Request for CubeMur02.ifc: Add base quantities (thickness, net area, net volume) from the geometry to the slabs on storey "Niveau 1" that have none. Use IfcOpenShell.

First a look at what the model holds.

```python
import ifcopenshell
import ifcopenshell.util.element
import ifcopenshell.util.unit

model = ifcopenshell.open("CubeMur02.ifc")
print(model.schema)
for unit_type in ("LENGTHUNIT", "AREAUNIT", "VOLUMEUNIT"):
    print(unit_type, ifcopenshell.util.unit.calculate_unit_scale(model, unit_type))
storey = next(s for s in model.by_type("IfcBuildingStorey") if s.Name == "Niveau 1")
slabs = [e for e in ifcopenshell.util.element.get_decomposition(storey) if e.is_a("IfcSlab")]
for e in sorted(slabs, key=lambda e: e.id()):
    print(e.id(), e.is_a(), e.Name, list(ifcopenshell.util.element.get_psets(e, qtos_only=True)), sep=" | ")
```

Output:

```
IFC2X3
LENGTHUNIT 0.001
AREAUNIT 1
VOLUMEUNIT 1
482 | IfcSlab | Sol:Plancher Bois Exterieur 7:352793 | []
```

```python
import ifcopenshell
import ifcopenshell.api.pset
import ifcopenshell.geom
import ifcopenshell.util.element
import ifcopenshell.util.shape
import ifcopenshell.util.unit

model = ifcopenshell.open("CubeMur02.ifc")
unit_scale = ifcopenshell.util.unit.calculate_unit_scale(model)
area_scale = ifcopenshell.util.unit.calculate_unit_scale(model, "AREAUNIT")
volume_scale = ifcopenshell.util.unit.calculate_unit_scale(model, "VOLUMEUNIT")
settings = ifcopenshell.geom.settings()

storey = next(s for s in model.by_type("IfcBuildingStorey") if s.Name == "Niveau 1")
slabs = [e for e in ifcopenshell.util.element.get_decomposition(storey) if e.is_a("IfcSlab")]

for e in sorted(slabs, key=lambda e: e.id()):
    if ifcopenshell.util.element.get_psets(e, qtos_only=True, should_inherit=False):
        continue
    # Geometry comes back in metres, in the element's own axes.
    shape = ifcopenshell.geom.create_shape(settings, e)
    values = {
        "Width": ifcopenshell.util.shape.get_z(shape.geometry) / unit_scale,
        "NetArea": ifcopenshell.util.shape.get_footprint_area(shape.geometry) / area_scale,
        "NetVolume": ifcopenshell.util.shape.get_volume(shape.geometry) / volume_scale,
    }
    qto = ifcopenshell.api.pset.add_qto(model, product=e, name="BaseQuantities")
    ifcopenshell.api.pset.edit_qto(model, qto=qto, properties=values)
    print(e.id(), {k: round(v, 3) for k, v in values.items()})

model.write("CubeMur02-out.ifc")
```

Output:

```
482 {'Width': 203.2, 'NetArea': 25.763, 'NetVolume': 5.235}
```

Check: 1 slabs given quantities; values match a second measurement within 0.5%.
